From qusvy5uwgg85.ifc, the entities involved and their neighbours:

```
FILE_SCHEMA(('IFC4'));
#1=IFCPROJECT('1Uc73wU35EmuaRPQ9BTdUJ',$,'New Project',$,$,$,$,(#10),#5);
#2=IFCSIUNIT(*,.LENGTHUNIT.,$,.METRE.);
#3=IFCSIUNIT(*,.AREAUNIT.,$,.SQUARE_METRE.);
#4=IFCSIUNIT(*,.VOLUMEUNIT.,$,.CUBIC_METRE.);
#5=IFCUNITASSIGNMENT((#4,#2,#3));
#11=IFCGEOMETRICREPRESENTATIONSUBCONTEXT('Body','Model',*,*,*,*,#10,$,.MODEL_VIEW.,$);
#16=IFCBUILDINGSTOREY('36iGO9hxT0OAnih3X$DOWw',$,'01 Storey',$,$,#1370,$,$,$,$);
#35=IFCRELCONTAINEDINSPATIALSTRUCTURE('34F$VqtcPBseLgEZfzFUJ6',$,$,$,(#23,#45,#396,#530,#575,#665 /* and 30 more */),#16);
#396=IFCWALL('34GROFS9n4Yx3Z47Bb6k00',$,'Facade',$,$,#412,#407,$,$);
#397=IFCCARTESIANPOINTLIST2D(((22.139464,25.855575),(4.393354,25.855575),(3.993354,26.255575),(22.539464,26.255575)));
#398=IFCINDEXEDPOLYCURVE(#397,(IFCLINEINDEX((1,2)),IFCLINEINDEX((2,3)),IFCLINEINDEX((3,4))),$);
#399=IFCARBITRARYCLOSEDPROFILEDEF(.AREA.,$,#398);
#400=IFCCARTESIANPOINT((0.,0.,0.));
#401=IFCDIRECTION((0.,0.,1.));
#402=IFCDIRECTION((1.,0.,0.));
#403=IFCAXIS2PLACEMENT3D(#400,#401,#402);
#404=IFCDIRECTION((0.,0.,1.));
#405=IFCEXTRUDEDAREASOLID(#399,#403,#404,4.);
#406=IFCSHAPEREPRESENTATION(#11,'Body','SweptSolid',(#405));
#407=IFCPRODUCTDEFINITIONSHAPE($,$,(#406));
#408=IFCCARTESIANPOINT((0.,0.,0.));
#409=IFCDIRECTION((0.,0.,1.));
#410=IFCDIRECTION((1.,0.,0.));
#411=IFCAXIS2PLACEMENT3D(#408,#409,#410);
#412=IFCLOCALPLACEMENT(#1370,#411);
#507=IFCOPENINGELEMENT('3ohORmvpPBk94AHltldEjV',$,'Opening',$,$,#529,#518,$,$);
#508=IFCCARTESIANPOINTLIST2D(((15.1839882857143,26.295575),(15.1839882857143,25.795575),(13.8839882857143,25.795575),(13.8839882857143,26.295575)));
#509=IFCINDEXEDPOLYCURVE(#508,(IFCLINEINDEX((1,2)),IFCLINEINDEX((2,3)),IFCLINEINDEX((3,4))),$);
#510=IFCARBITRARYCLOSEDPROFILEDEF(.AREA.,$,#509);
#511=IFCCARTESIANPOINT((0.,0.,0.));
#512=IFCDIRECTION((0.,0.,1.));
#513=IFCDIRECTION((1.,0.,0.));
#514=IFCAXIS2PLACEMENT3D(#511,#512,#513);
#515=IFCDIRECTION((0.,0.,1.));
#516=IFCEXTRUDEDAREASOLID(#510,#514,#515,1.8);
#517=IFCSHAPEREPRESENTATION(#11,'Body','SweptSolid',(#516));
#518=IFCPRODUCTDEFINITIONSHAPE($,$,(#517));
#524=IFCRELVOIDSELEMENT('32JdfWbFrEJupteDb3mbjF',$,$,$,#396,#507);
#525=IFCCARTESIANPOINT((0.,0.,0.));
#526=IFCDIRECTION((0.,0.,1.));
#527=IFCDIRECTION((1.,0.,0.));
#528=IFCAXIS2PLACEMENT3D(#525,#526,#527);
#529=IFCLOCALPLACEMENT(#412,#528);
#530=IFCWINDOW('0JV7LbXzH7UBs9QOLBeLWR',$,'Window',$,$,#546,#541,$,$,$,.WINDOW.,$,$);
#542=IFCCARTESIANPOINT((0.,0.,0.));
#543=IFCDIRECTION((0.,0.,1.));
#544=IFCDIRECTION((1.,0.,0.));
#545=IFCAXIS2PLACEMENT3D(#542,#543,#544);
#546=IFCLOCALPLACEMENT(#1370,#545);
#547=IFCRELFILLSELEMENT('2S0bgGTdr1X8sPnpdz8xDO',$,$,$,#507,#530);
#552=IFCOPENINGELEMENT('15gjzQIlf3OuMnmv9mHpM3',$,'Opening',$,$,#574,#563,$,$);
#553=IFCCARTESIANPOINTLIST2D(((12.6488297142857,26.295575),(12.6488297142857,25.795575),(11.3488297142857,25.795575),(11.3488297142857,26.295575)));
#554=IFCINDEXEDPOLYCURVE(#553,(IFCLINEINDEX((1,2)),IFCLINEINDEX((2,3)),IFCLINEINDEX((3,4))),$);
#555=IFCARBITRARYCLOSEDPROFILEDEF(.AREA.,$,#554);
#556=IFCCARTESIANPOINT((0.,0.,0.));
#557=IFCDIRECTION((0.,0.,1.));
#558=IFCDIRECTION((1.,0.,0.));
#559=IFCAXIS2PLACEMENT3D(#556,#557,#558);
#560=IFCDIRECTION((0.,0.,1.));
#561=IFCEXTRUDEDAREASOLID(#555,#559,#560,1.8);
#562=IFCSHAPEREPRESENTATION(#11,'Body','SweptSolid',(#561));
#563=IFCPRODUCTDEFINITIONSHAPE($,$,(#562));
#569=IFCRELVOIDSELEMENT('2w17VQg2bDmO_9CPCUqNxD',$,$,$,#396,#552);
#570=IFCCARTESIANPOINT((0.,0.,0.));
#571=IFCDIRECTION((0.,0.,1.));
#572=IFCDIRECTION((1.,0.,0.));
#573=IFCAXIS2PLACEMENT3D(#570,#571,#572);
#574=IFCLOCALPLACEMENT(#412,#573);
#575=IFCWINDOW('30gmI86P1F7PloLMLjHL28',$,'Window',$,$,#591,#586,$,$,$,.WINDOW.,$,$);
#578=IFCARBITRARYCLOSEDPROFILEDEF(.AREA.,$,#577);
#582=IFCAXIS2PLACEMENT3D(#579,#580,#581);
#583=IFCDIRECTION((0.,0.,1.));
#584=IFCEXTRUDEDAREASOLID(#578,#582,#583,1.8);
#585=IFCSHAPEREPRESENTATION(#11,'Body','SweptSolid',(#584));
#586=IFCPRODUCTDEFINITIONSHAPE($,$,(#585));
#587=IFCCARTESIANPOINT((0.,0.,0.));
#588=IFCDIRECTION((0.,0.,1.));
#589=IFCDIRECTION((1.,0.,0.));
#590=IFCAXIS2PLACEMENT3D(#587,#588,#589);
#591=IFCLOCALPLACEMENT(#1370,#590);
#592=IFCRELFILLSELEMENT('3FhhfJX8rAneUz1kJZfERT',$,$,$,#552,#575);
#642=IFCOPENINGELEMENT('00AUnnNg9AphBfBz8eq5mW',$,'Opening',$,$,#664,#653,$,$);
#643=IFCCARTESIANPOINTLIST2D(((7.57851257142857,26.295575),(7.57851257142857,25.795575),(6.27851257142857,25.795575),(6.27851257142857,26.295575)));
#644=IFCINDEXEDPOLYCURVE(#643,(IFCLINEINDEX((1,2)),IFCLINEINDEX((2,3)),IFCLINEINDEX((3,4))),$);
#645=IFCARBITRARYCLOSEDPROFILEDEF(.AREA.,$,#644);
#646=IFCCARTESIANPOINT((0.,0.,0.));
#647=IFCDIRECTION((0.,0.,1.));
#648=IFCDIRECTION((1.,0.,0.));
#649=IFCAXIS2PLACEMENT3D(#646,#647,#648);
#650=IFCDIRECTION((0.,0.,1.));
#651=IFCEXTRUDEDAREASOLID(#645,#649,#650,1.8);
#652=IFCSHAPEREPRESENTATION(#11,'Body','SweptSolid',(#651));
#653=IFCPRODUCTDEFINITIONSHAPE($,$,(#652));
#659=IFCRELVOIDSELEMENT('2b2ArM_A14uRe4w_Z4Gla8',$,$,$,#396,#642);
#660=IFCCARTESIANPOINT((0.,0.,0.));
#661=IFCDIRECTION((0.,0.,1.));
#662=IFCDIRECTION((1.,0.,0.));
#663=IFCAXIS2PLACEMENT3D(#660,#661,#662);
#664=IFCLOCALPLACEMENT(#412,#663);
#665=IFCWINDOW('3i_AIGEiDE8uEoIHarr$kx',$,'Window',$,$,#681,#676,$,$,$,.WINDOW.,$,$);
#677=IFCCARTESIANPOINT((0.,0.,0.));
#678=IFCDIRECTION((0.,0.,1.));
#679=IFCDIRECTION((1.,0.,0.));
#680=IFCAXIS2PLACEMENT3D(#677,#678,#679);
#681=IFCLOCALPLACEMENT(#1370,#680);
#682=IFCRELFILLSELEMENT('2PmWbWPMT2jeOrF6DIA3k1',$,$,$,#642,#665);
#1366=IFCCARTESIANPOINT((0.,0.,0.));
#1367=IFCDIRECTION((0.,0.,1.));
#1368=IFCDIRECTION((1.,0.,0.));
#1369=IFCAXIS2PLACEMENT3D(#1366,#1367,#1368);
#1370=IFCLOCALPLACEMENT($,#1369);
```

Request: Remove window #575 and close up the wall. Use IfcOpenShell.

```python
import ifcopenshell
import ifcopenshell.api.feature
import ifcopenshell.api.root
import ifcopenshell.geom
import ifcopenshell.util.shape

model = ifcopenshell.open("qusvy5uwgg85.ifc")
settings = ifcopenshell.geom.settings()


def volume(element):
    """Net volume in cubic metres, openings subtracted."""
    shape = ifcopenshell.geom.create_shape(settings, element)
    return ifcopenshell.util.shape.get_volume(shape.geometry)


window = model.by_guid("30gmI86P1F7PloLMLjHL28")
opening = window.FillsVoids[0].RelatingOpeningElement
wall = opening.VoidsElements[0].RelatingBuildingElement
before = volume(wall)

ifcopenshell.api.root.remove_product(model, product=window)
ifcopenshell.api.feature.remove_feature(model, feature=opening)

after = volume(wall)

print(f"wall volume {before:.3f} -> {after:.3f} m3")

model.write("qusvy5uwgg85_v2.ifc")
```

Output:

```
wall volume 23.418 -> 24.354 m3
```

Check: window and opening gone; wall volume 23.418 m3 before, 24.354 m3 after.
